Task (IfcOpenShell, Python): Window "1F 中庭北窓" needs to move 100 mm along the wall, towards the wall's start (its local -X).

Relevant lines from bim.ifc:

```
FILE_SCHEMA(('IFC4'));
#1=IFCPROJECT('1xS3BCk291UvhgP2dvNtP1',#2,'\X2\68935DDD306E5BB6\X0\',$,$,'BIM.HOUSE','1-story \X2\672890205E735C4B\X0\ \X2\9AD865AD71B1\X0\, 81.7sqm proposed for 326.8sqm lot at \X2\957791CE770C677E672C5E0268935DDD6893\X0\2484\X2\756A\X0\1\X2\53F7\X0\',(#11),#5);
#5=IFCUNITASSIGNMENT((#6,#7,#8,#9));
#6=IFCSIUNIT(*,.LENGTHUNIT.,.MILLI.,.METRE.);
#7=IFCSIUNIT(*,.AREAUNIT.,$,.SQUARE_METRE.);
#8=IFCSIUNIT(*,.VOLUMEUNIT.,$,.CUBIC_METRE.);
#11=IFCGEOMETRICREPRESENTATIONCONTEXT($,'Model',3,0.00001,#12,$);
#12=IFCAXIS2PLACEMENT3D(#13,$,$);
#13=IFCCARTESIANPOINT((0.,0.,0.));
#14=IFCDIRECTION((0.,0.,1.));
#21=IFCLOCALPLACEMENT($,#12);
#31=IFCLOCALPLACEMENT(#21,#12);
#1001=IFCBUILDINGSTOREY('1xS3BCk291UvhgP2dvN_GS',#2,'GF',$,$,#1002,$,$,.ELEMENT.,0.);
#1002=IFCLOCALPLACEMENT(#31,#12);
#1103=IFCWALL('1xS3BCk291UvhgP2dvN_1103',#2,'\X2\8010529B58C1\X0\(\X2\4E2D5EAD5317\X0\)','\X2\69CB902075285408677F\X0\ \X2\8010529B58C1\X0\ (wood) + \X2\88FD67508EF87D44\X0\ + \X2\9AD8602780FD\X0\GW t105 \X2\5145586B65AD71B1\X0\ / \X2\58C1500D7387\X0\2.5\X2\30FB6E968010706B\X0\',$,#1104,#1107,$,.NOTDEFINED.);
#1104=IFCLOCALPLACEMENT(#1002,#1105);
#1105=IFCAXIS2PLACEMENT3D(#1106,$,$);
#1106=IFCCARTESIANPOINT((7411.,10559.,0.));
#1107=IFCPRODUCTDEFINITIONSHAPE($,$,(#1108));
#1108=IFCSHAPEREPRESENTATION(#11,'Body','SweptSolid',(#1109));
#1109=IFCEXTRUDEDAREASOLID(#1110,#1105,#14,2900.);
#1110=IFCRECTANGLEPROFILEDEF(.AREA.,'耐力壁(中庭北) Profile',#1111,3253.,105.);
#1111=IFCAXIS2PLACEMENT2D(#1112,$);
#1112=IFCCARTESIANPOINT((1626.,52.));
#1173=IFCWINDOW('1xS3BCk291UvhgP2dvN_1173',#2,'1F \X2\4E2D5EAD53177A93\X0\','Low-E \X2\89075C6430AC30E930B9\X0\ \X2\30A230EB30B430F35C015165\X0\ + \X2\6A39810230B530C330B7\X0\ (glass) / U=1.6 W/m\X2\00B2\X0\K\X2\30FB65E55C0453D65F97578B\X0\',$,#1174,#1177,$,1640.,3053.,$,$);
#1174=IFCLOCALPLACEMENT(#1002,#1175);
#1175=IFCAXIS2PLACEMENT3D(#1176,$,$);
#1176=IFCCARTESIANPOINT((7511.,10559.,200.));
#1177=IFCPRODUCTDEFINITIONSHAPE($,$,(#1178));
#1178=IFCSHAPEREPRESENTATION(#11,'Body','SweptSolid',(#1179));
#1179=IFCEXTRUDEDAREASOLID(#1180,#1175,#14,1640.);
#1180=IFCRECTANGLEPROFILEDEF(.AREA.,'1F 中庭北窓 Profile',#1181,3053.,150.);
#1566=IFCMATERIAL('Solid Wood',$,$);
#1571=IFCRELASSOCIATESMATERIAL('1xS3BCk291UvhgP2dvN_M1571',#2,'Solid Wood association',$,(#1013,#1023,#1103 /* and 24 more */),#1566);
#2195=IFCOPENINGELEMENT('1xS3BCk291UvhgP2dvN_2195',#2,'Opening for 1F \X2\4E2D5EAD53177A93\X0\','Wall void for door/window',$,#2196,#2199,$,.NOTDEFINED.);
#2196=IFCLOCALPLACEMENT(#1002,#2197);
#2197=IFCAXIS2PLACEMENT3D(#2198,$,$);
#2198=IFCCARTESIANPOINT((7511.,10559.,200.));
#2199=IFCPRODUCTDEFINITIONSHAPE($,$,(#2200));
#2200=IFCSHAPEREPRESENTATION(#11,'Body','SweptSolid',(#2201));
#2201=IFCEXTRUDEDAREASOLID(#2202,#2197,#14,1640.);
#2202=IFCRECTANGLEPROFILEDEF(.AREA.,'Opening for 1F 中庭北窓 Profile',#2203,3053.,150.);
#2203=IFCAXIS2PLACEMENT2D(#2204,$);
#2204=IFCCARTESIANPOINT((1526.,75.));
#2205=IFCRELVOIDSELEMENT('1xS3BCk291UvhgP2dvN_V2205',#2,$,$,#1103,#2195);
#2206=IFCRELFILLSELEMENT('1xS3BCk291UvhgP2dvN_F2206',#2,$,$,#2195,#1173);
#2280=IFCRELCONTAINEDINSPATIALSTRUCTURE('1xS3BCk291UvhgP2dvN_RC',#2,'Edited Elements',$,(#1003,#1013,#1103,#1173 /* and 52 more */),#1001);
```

```python
import ifcopenshell
import ifcopenshell.api.geometry
import ifcopenshell.util.placement

model = ifcopenshell.open("bim.ifc")

window = model.by_id(1173)
opening = window.FillsVoids[0].RelatingOpeningElement
wall = opening.VoidsElements[0].RelatingBuildingElement

wall_matrix = ifcopenshell.util.placement.get_local_placement(wall.ObjectPlacement)
shift = wall_matrix[:3, 0] * -100.0
before = ifcopenshell.util.placement.get_local_placement(window.ObjectPlacement)[:3, 3].copy()

# The window is not placed relative to its opening, so move both.
for product in (opening, window):
    matrix = ifcopenshell.util.placement.get_local_placement(product.ObjectPlacement)
    matrix[:3, 3] += shift
    ifcopenshell.api.geometry.edit_object_placement(model, product=product, matrix=matrix, is_si=False)

after = ifcopenshell.util.placement.get_local_placement(window.ObjectPlacement)[:3, 3]
print("window moved by", (after - before).round(3) + 0.0)

model.write("bim-out.ifc")
```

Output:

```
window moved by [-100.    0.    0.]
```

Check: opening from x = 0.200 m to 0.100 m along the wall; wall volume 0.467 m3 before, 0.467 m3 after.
